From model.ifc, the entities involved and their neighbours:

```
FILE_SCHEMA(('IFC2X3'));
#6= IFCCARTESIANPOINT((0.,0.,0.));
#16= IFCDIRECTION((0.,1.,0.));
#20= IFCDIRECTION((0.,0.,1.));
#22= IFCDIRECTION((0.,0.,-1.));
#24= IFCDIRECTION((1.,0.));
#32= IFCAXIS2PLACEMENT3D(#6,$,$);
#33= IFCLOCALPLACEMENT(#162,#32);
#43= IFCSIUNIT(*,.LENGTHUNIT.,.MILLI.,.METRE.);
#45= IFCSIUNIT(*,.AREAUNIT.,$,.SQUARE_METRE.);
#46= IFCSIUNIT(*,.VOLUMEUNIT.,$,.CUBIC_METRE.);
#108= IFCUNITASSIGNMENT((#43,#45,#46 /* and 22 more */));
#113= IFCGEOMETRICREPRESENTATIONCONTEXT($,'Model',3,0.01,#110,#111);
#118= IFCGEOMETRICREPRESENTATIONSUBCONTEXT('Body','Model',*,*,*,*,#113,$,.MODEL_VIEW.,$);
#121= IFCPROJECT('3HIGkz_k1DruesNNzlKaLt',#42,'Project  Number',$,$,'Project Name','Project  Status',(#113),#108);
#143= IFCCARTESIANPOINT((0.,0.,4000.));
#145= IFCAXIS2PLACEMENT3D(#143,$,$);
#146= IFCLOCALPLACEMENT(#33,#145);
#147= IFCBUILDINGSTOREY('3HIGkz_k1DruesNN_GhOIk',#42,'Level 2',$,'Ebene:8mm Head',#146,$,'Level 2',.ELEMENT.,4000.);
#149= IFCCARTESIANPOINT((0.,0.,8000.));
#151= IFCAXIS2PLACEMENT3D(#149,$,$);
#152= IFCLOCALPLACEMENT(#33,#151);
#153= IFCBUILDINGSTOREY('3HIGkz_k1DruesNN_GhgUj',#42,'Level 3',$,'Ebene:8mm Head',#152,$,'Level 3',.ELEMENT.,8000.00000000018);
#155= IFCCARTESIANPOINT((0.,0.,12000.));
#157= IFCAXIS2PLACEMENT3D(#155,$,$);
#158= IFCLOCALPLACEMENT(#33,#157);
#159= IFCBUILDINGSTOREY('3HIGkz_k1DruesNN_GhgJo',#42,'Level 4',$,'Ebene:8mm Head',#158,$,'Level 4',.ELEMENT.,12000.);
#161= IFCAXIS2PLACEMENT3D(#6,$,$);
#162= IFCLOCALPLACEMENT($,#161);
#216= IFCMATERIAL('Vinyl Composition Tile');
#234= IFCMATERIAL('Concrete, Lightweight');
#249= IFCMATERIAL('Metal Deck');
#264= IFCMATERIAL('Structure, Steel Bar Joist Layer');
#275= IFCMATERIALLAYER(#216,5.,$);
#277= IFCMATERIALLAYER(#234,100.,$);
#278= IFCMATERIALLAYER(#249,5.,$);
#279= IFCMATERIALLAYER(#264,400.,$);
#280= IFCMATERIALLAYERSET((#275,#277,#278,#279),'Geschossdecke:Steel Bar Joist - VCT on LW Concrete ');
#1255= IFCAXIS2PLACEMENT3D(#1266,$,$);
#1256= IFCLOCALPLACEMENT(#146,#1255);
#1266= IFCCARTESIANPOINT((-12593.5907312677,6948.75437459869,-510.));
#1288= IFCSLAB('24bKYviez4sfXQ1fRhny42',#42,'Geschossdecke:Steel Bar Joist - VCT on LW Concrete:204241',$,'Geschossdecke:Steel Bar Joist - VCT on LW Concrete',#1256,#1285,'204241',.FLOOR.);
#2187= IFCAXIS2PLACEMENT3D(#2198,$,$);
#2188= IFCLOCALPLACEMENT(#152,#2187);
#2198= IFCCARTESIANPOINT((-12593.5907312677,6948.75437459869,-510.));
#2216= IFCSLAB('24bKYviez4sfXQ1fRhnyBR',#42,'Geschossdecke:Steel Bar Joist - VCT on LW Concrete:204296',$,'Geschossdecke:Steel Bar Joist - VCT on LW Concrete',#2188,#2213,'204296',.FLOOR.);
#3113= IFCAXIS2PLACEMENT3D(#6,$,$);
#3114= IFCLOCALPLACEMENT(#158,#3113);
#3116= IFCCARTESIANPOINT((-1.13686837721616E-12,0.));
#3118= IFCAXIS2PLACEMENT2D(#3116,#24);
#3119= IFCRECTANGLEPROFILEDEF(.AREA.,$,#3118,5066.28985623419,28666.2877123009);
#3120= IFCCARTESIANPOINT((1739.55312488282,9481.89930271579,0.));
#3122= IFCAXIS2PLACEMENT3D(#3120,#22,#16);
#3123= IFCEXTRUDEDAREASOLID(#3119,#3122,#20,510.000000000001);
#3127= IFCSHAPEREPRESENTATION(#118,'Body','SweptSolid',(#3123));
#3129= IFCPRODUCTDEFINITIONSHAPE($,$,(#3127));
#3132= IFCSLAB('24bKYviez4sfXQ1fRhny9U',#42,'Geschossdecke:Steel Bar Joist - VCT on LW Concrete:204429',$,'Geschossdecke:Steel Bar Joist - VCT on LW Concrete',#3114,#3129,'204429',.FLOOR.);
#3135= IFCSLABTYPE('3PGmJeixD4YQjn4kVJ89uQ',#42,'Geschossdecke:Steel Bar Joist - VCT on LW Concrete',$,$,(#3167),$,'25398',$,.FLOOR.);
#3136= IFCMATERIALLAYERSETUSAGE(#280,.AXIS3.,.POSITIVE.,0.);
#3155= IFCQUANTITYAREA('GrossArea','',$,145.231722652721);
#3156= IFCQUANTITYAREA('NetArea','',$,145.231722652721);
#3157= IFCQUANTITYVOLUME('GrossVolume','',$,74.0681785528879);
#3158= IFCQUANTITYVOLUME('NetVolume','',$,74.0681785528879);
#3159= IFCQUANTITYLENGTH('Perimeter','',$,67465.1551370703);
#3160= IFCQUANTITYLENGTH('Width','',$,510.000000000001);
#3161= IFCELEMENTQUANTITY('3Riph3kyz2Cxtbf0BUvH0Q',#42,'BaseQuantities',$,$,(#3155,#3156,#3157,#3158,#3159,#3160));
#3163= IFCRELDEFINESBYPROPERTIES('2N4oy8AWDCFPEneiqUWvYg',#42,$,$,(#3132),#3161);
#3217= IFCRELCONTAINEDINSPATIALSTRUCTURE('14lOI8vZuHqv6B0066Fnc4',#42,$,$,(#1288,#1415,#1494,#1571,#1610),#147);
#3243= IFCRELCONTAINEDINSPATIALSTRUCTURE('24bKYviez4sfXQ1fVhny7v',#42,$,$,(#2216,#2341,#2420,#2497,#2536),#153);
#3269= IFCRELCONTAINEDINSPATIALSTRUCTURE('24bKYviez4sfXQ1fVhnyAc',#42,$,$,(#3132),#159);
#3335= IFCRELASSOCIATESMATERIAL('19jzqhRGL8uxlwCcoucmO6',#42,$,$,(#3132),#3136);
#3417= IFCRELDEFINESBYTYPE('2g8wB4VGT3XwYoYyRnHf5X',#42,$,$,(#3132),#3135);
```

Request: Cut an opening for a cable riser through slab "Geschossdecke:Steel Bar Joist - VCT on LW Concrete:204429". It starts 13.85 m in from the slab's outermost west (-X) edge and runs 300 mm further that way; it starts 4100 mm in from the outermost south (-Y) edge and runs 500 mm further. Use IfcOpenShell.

```python
import numpy as np
import ifcopenshell
import ifcopenshell.api.feature
import ifcopenshell.api.geometry
import ifcopenshell.api.pset
import ifcopenshell.api.root
import ifcopenshell.geom
import ifcopenshell.util.element
import ifcopenshell.util.placement
import ifcopenshell.util.representation
import ifcopenshell.util.shape
import ifcopenshell.util.unit

model = ifcopenshell.open("model.ifc")
unit_scale = ifcopenshell.util.unit.calculate_unit_scale(model)
area_scale = ifcopenshell.util.unit.calculate_unit_scale(model, "AREAUNIT")
volume_scale = ifcopenshell.util.unit.calculate_unit_scale(model, "VOLUMEUNIT")
settings = ifcopenshell.geom.settings()


def volume(element):
    """Net volume in cubic metres, openings subtracted."""
    shape = ifcopenshell.geom.create_shape(settings, element)
    return ifcopenshell.util.shape.get_volume(shape.geometry)


slab = model.by_guid("24bKYviez4sfXQ1fRhny9U")
before = volume(slab)

# Extent in the slab's own axes, in metres. The edges named are its -X and -Y sides.
slab_shape = ifcopenshell.geom.create_shape(settings, slab)
vertices = ifcopenshell.util.shape.get_vertices(slab_shape.geometry)
x_min, y_min, bottom = vertices.min(axis=0)
top = vertices[:, 2].max()

opening = ifcopenshell.api.root.create_entity(model, ifc_class="IfcOpeningElement", name="Cable riser opening")
context = ifcopenshell.util.representation.get_context(model, "Model", "Body", "MODEL_VIEW")
width, depth = 0.3, 0.5
outline = [(0.0, 0.0), (width, 0.0), (width, depth), (0.0, depth), (0.0, 0.0)]
# Overshoot both faces by 50 mm so the cut is clean.
shape = ifcopenshell.api.geometry.add_slab_representation(
    model, context=context, depth=top - bottom + 0.1, polyline=outline
)
ifcopenshell.api.geometry.assign_representation(model, product=opening, representation=shape)

matrix = ifcopenshell.util.placement.get_local_placement(slab.ObjectPlacement)
matrix[:, 3] = matrix @ np.append(np.array([x_min + 13.85, y_min + 4.1, bottom - 0.05]) / unit_scale, 1.0)
ifcopenshell.api.geometry.edit_object_placement(model, product=opening, matrix=matrix, is_si=False)
ifcopenshell.api.feature.add_feature(model, feature=opening, element=slab)

after = volume(slab)

# Update the slab's stored quantities.
qto = model.by_id(ifcopenshell.util.element.get_pset(slab, "BaseQuantities", should_inherit=False)["id"])
ifcopenshell.api.pset.edit_qto(model, qto=qto, properties={
    "NetArea": after / (top - bottom) / area_scale,
    "NetVolume": after / volume_scale,
})

print(f"slab volume {before:.3f} -> {after:.3f} m3")

model.write("model-out.ifc")
```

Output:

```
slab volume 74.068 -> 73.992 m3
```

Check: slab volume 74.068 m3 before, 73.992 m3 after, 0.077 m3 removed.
